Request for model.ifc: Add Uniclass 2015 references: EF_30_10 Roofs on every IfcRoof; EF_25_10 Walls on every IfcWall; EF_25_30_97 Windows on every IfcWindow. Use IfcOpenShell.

First a look at what the model holds.

```python
import ifcopenshell

model = ifcopenshell.open("model.ifc")
print(model.schema)
print("classifications:", [c.Name for c in model.by_type("IfcClassification")])
for ifc_class in ("IfcDoor", "IfcRoof", "IfcStair", "IfcWall", "IfcWindow"):
    print(ifc_class, len(model.by_type(ifc_class)))
```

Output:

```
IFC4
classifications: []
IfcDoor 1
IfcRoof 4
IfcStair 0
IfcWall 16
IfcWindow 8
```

```python
import ifcopenshell
import ifcopenshell.api.classification

model = ifcopenshell.open("model.ifc")

system = ifcopenshell.api.classification.add_classification(model, classification="Uniclass 2015")

codes = {
    "IfcRoof": ("EF_30_10", "Roofs"),
    "IfcWall": ("EF_25_10", "Walls"),
    "IfcWindow": ("EF_25_30_97", "Windows"),
}
for ifc_class, (code, name) in codes.items():
    products = model.by_type(ifc_class)
    ifcopenshell.api.classification.add_reference(
        model, products=products, classification=system, identification=code, name=name
    )
    print(code, len(products))

model.write("model-out.ifc")
```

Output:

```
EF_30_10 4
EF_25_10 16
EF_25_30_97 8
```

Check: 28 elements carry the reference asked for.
